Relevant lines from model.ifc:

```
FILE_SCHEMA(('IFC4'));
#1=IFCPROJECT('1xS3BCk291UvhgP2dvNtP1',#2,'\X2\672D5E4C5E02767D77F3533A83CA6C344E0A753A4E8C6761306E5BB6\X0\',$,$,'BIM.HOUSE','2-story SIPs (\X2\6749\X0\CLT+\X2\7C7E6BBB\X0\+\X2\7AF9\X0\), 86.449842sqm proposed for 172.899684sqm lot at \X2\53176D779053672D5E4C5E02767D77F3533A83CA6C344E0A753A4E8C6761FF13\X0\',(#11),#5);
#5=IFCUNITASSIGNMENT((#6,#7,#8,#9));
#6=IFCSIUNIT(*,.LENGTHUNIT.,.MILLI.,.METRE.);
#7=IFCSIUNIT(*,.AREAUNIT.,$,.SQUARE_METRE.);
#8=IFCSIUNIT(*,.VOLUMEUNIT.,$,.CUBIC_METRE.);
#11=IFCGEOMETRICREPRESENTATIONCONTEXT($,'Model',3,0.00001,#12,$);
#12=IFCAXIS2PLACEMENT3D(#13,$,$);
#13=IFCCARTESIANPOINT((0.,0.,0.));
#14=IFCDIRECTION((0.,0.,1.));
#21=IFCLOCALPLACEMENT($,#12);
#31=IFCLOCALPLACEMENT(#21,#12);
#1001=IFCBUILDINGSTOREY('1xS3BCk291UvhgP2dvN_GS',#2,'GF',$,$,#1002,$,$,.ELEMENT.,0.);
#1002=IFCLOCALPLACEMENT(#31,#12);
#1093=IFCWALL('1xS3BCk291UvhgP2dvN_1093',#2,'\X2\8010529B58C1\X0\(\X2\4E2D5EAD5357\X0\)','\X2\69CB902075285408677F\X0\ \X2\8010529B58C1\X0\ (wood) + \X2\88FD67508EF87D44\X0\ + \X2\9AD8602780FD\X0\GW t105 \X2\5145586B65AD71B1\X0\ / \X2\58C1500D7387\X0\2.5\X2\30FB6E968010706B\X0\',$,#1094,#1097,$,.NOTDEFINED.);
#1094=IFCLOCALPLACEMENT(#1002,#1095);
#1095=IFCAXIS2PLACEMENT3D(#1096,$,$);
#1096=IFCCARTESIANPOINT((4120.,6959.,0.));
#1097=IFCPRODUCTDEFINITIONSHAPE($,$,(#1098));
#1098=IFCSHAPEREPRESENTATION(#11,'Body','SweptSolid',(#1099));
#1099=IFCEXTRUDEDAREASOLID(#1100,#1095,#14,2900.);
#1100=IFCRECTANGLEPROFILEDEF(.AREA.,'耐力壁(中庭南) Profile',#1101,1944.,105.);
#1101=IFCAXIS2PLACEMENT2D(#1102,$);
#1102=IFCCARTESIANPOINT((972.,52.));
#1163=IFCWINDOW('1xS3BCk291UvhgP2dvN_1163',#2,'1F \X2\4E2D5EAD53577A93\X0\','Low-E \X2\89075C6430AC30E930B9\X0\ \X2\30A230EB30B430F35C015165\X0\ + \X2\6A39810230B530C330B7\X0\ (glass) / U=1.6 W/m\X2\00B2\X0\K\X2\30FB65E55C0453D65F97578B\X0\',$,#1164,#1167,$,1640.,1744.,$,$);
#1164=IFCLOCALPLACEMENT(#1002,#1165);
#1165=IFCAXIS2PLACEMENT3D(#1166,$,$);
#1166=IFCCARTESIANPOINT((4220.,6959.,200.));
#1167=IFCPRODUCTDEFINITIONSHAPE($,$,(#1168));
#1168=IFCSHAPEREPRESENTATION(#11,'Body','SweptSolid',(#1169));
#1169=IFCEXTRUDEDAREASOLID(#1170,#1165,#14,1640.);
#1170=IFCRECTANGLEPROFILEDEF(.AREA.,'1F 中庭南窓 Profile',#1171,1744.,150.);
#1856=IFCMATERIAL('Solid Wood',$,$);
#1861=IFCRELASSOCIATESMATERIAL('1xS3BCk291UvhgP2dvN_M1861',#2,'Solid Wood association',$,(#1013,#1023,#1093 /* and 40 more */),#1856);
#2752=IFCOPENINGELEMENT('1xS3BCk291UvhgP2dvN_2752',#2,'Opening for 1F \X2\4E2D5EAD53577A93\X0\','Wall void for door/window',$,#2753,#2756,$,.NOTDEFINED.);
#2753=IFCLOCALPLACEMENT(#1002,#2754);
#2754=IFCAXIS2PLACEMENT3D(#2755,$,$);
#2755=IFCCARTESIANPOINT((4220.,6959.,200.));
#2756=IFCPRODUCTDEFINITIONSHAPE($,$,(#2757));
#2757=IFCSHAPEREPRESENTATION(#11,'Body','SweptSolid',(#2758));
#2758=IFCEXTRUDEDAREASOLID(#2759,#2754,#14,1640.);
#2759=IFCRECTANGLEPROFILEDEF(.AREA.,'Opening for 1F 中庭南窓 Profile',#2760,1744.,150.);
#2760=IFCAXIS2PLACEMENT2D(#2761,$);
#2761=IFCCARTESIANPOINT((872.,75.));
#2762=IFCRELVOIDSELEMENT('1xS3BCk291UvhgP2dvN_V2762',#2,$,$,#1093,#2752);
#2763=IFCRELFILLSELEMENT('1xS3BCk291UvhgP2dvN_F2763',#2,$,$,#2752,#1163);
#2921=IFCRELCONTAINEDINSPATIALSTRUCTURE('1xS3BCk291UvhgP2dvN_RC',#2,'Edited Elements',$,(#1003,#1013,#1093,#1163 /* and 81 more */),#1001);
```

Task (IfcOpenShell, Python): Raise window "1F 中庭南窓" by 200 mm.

```python
import numpy as np
import ifcopenshell
import ifcopenshell.api.geometry
import ifcopenshell.util.placement
import ifcopenshell.util.unit

model = ifcopenshell.open("model.ifc")
unit_scale = ifcopenshell.util.unit.calculate_unit_scale(model)

window = model.by_id(1163)
opening = window.FillsVoids[0].RelatingOpeningElement
dz = 0.2 / unit_scale

shift = np.array([0.0, 0.0, dz])
# The window is not placed relative to its opening, so move both.
for product in (opening, window):
    matrix = ifcopenshell.util.placement.get_local_placement(product.ObjectPlacement)
    matrix[:3, 3] += shift
    ifcopenshell.api.geometry.edit_object_placement(model, product=product, matrix=matrix, is_si=False)

print(f"moved by {dz * unit_scale:+.3f} m")

model.write("model_edited.ifc")
```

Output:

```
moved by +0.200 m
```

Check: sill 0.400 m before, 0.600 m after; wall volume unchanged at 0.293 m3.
